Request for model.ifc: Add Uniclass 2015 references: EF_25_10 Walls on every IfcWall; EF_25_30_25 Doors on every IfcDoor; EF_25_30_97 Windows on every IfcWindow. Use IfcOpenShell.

First a look at what the model holds.

```python
import ifcopenshell

model = ifcopenshell.open("model.ifc")
print(model.schema)
print("classifications:", [c.Name for c in model.by_type("IfcClassification")])
for ifc_class in ("IfcDoor", "IfcRoof", "IfcStair", "IfcWall", "IfcWindow"):
    print(ifc_class, len(model.by_type(ifc_class)))
```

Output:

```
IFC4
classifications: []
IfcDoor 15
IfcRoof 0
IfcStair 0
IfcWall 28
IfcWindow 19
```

```python
import ifcopenshell
import ifcopenshell.api.classification

model = ifcopenshell.open("model.ifc")

system = ifcopenshell.api.classification.add_classification(model, classification="Uniclass 2015")

codes = {
    "IfcWall": ("EF_25_10", "Walls"),
    "IfcDoor": ("EF_25_30_25", "Doors"),
    "IfcWindow": ("EF_25_30_97", "Windows"),
}
for ifc_class, (code, name) in codes.items():
    products = model.by_type(ifc_class)
    ifcopenshell.api.classification.add_reference(
        model, products=products, classification=system, identification=code, name=name
    )
    print(code, len(products))

model.write("model_edited.ifc")
```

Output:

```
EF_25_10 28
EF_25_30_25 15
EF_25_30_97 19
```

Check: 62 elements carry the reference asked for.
